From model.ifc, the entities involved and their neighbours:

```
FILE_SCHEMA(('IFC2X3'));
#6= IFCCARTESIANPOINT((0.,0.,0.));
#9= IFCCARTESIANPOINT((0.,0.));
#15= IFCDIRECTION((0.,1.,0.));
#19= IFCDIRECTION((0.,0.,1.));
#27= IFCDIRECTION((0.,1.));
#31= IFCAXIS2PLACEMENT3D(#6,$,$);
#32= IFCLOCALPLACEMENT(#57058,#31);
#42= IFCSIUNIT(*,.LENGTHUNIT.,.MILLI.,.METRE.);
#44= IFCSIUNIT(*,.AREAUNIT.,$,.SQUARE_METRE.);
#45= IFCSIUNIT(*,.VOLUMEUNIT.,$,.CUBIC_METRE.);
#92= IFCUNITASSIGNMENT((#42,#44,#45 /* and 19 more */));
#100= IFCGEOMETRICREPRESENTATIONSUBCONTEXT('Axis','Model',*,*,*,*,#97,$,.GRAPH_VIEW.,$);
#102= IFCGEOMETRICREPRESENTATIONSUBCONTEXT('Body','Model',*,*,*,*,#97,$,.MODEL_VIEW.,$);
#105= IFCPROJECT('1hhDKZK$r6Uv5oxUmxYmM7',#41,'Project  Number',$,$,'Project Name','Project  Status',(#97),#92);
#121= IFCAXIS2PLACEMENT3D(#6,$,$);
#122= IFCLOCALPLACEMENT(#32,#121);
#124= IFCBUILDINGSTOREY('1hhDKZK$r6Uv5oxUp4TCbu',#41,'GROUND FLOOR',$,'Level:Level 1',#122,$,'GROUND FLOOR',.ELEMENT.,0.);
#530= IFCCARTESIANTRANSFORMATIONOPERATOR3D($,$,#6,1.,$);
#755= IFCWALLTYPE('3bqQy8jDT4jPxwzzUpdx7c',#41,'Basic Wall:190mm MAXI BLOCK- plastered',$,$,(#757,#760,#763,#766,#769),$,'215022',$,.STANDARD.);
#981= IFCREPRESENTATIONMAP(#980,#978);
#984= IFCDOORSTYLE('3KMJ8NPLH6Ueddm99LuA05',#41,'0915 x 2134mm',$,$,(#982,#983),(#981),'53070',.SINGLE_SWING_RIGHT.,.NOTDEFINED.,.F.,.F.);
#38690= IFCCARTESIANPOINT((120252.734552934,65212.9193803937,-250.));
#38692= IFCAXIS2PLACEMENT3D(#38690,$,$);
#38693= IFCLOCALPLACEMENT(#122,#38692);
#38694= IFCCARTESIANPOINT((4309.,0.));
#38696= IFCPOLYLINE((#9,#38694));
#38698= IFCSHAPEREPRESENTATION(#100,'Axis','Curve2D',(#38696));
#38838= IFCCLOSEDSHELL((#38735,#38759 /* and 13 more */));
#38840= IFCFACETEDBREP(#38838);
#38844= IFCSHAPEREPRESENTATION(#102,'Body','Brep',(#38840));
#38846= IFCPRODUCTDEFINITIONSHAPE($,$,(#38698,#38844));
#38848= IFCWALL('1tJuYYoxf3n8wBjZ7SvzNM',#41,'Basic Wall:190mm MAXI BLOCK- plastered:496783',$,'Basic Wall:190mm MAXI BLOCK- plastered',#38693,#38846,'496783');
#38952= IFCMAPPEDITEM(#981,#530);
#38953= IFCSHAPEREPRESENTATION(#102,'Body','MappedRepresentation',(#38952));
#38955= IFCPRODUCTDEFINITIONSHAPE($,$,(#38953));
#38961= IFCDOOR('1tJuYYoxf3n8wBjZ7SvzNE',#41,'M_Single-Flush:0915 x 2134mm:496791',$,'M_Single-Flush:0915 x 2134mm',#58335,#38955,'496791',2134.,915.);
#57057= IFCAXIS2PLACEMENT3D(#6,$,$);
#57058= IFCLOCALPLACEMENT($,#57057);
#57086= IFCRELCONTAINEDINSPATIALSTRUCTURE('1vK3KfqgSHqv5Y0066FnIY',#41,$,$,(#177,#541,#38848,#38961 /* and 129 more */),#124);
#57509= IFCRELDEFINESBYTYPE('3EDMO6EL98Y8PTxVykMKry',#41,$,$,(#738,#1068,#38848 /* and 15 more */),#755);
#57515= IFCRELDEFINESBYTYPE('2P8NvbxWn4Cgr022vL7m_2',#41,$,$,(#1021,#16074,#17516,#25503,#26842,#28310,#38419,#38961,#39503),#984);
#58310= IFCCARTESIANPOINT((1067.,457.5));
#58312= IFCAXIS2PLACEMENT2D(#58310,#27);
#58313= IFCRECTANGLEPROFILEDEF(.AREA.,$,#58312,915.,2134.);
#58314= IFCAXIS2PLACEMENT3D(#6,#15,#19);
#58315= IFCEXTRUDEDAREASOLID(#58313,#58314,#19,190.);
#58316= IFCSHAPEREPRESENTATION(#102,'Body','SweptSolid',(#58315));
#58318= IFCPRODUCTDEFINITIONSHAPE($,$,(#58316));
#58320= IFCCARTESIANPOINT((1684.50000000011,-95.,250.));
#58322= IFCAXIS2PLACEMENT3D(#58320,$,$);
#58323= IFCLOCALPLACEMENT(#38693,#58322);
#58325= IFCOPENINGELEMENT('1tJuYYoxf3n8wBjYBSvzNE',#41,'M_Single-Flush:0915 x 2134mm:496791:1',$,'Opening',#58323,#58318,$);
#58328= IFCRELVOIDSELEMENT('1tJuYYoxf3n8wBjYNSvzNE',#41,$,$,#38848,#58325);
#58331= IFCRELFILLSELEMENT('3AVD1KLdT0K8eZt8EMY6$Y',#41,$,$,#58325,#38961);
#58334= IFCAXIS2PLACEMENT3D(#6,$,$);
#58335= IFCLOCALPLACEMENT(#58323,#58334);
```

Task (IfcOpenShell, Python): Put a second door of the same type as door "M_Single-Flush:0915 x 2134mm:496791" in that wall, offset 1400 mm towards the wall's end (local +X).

```python
import ifcopenshell
import ifcopenshell.api.feature
import ifcopenshell.api.geometry
import ifcopenshell.api.root
import ifcopenshell.geom
import ifcopenshell.util.element
import ifcopenshell.util.placement
import ifcopenshell.util.shape

model = ifcopenshell.open("model.ifc")
settings = ifcopenshell.geom.settings()


def volume(element):
    """Net volume in cubic metres, openings subtracted."""
    shape = ifcopenshell.geom.create_shape(settings, element)
    return ifcopenshell.util.shape.get_volume(shape.geometry)


def reuse_history(source, copy):
    """copy_class also copies each property set's owner history, people and application; keep the originals."""
    for rel in copy.IsDefinedBy:
        if rel.is_a("IfcRelDefinesByProperties") and (history := rel.RelatingPropertyDefinition.OwnerHistory):
            rel.RelatingPropertyDefinition.OwnerHistory = source.OwnerHistory
            ifcopenshell.util.element.remove_deep2(model, history)


door = model.by_guid("1tJuYYoxf3n8wBjZ7SvzNE")
opening = door.FillsVoids[0].RelatingOpeningElement
wall = opening.VoidsElements[0].RelatingBuildingElement
before = volume(wall)
shift = ifcopenshell.util.placement.get_local_placement(wall.ObjectPlacement)[:3, 0] * 1400.0

# copy_class copies the void relationship, type, container and properties, but no geometry.
new_opening = ifcopenshell.api.root.copy_class(model, product=opening)
new_opening.Representation = ifcopenshell.util.element.copy_deep(
    model, opening.Representation, exclude=["IfcGeometricRepresentationContext", "IfcRepresentationMap"]
)
new_opening.Name = "M_Single-Flush:0915 x 2134mm"
new_door = ifcopenshell.api.root.copy_class(model, product=door)
new_door.Representation = ifcopenshell.util.element.copy_deep(
    model, door.Representation, exclude=["IfcGeometricRepresentationContext", "IfcRepresentationMap"]
)
new_door.Name = "M_Single-Flush:0915 x 2134mm"
new_door.Tag = None
reuse_history(door, new_door)
fills = ifcopenshell.api.feature.add_filling(model, opening=new_opening, element=new_door)
fills.OwnerHistory = new_door.OwnerHistory  # required in IFC2X3

for old, new in ((opening, new_opening), (door, new_door)):
    matrix = ifcopenshell.util.placement.get_local_placement(old.ObjectPlacement)
    matrix[:3, 3] += shift
    ifcopenshell.api.geometry.edit_object_placement(model, product=new, matrix=matrix, is_si=False)

after = volume(wall)

print(f"wall volume {before:.3f} -> {after:.3f} m3")

model.write("model_updated.ifc")
```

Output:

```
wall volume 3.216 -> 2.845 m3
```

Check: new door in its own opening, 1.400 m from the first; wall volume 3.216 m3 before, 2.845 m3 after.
